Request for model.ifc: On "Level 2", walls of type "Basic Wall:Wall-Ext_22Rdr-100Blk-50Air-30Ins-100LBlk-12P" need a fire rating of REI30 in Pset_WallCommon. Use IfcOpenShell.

First a look at what the model holds.

```python
import ifcopenshell
import ifcopenshell.util.element

model = ifcopenshell.open("model.ifc")
print(model.schema)
storey = next(s for s in model.by_type("IfcBuildingStorey") if s.Name == "Level 2")
walls = [e for e in ifcopenshell.util.element.get_decomposition(storey) if e.is_a("IfcWall")]
seen = {}
for e in walls:
    element_type = ifcopenshell.util.element.get_type(e)
    key = (element_type.Name if element_type != e and element_type else None, ifcopenshell.util.element.get_pset(e, "Pset_WallCommon", "FireRating"))
    seen[key] = seen.get(key, 0) + 1
for (name, value), count in sorted(seen.items(), key=str):
    print(count, "x", name, "|", value)
```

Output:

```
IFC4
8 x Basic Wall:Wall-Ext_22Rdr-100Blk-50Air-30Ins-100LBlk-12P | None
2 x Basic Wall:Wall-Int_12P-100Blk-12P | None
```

```python
import ifcopenshell
import ifcopenshell.api.pset
import ifcopenshell.util.element

model = ifcopenshell.open("model.ifc")

storey = next(s for s in model.by_type("IfcBuildingStorey") if s.Name == "Level 2")
walls = [e for e in ifcopenshell.util.element.get_decomposition(storey) if e.is_a("IfcWall")]

count = 0
for e in walls:
    element_type = ifcopenshell.util.element.get_type(e)
    if element_type in (None, e) or element_type.Name != "Basic Wall:Wall-Ext_22Rdr-100Blk-50Air-30Ins-100LBlk-12P":
        continue
    # add_pset returns the element's existing set when there is one.
    pset = ifcopenshell.api.pset.add_pset(model, product=e, name="Pset_WallCommon")
    ifcopenshell.api.pset.edit_pset(model, pset=pset, properties={"FireRating": "REI30"})
    count += 1

print(count, "walls updated")

model.write("model_updated.ifc")
```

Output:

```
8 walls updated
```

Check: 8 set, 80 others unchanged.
